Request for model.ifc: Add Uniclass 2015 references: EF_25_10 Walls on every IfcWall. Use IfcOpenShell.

First a look at what the model holds.

```python
import ifcopenshell

model = ifcopenshell.open("model.ifc")
print(model.schema)
print("classifications:", [c.Name for c in model.by_type("IfcClassification")])
for ifc_class in ("IfcDoor", "IfcRoof", "IfcStair", "IfcWall", "IfcWindow"):
    print(ifc_class, len(model.by_type(ifc_class)))
```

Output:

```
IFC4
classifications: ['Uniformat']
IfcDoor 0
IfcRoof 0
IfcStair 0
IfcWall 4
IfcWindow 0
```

```python
import ifcopenshell
import ifcopenshell.api.classification

model = ifcopenshell.open("model.ifc")

system = ifcopenshell.api.classification.add_classification(model, classification="Uniclass 2015")

codes = {
    "IfcWall": ("EF_25_10", "Walls"),
}
for ifc_class, (code, name) in codes.items():
    products = model.by_type(ifc_class)
    ifcopenshell.api.classification.add_reference(
        model, products=products, classification=system, identification=code, name=name
    )
    print(code, len(products))

model.write("model_edited.ifc")
```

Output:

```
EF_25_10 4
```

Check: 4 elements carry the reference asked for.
